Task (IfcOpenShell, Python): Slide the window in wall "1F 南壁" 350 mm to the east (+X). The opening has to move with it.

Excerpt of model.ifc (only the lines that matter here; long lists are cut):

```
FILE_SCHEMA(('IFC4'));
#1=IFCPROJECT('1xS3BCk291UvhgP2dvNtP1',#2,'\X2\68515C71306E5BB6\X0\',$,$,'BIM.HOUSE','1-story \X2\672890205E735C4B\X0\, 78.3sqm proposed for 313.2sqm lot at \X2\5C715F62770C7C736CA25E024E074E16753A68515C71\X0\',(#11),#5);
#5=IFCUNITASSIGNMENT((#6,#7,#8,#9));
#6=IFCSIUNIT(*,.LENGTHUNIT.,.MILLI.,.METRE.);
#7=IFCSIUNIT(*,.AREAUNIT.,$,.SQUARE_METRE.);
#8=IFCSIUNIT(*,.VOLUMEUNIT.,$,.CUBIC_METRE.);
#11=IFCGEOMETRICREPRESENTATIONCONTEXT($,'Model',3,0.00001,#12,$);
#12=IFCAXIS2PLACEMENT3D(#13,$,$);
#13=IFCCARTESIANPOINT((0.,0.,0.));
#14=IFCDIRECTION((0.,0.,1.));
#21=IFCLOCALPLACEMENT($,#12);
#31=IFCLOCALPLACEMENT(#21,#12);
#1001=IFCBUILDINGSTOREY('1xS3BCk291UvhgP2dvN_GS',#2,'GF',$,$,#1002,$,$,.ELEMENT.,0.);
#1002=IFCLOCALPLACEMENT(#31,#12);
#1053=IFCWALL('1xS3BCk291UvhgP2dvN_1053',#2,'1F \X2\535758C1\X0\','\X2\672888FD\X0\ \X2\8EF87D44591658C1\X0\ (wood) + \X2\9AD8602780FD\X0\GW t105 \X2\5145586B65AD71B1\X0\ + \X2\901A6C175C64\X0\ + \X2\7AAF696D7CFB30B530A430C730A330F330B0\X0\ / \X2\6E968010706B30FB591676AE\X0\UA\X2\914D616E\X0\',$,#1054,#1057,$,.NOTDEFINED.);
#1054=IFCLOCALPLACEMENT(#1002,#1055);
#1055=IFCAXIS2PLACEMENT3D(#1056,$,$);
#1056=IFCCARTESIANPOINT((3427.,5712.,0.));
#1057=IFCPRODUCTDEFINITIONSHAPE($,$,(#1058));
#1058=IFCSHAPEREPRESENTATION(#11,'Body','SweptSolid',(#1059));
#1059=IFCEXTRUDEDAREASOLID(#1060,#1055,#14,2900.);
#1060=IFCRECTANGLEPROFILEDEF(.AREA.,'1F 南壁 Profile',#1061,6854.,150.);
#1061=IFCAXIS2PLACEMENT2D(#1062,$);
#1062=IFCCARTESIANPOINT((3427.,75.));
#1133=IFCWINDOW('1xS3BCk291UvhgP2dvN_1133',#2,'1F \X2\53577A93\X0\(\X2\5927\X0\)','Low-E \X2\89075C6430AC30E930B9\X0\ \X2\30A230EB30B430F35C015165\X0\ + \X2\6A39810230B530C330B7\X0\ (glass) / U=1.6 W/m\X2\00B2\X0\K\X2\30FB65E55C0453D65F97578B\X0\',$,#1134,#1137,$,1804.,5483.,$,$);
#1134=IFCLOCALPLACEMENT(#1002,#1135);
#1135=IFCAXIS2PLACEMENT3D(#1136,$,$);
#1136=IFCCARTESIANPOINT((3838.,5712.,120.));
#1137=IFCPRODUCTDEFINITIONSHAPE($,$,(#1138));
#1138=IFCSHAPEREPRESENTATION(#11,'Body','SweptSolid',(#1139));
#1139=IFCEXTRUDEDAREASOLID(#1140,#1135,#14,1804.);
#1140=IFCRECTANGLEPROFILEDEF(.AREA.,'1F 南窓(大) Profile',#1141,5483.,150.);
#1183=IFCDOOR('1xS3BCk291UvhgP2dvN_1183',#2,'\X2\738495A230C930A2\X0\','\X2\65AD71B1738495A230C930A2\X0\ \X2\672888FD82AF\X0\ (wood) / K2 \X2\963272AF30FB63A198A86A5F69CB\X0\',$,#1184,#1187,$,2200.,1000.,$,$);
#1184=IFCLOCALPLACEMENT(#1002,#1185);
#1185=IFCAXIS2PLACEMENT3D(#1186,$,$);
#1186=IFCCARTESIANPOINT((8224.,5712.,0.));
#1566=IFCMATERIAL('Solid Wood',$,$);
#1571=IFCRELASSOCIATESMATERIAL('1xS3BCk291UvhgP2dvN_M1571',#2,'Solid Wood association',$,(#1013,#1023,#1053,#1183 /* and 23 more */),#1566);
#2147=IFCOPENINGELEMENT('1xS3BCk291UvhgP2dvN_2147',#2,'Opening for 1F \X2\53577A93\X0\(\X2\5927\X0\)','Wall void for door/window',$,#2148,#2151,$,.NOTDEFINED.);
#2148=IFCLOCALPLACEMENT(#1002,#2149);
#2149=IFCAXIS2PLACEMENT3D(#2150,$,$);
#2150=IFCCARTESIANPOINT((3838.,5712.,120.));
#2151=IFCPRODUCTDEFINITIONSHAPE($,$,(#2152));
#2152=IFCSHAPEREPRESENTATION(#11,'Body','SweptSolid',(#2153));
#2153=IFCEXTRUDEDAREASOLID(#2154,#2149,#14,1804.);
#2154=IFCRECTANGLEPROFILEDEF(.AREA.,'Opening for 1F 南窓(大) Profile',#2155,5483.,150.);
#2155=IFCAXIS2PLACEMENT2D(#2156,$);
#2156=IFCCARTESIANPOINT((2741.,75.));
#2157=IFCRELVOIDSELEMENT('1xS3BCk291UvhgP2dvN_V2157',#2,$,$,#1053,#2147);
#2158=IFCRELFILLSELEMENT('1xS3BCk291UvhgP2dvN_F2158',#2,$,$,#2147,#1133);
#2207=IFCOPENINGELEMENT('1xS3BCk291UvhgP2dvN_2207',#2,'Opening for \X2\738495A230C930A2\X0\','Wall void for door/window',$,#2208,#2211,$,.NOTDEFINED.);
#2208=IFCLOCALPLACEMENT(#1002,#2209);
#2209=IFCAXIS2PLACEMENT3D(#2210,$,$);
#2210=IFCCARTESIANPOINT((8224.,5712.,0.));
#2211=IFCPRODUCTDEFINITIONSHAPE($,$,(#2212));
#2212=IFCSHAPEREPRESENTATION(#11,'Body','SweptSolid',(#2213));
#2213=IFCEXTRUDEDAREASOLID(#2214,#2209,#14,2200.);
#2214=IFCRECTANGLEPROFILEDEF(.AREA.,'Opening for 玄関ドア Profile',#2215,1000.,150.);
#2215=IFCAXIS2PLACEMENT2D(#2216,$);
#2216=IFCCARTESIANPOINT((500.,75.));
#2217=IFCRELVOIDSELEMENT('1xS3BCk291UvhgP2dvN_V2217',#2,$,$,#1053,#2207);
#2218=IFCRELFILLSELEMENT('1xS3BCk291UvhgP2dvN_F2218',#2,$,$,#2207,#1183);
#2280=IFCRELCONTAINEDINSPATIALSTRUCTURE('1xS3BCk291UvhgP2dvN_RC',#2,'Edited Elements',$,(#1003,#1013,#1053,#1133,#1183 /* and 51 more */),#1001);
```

```python
import ifcopenshell
import ifcopenshell.api.geometry
import ifcopenshell.util.placement
import ifcopenshell.util.unit

model = ifcopenshell.open("model.ifc")
unit_scale = ifcopenshell.util.unit.calculate_unit_scale(model)

window = model.by_guid("1xS3BCk291UvhgP2dvN_1133")
opening = window.FillsVoids[0].RelatingOpeningElement
wall = opening.VoidsElements[0].RelatingBuildingElement

wall_matrix = ifcopenshell.util.placement.get_local_placement(wall.ObjectPlacement)
shift = wall_matrix[:3, 0] * 0.35 / unit_scale
before = ifcopenshell.util.placement.get_local_placement(window.ObjectPlacement)[:3, 3].copy()

# The window is not placed relative to its opening, so move both.
for product in (opening, window):
    matrix = ifcopenshell.util.placement.get_local_placement(product.ObjectPlacement)
    matrix[:3, 3] += shift
    ifcopenshell.api.geometry.edit_object_placement(model, product=product, matrix=matrix, is_si=False)

after = ifcopenshell.util.placement.get_local_placement(window.ObjectPlacement)[:3, 3]
print("window moved by", (after - before).round(3) + 0.0)

model.write("model_updated.ifc")
```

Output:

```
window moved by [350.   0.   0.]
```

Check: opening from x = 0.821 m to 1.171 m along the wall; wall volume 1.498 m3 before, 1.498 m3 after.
